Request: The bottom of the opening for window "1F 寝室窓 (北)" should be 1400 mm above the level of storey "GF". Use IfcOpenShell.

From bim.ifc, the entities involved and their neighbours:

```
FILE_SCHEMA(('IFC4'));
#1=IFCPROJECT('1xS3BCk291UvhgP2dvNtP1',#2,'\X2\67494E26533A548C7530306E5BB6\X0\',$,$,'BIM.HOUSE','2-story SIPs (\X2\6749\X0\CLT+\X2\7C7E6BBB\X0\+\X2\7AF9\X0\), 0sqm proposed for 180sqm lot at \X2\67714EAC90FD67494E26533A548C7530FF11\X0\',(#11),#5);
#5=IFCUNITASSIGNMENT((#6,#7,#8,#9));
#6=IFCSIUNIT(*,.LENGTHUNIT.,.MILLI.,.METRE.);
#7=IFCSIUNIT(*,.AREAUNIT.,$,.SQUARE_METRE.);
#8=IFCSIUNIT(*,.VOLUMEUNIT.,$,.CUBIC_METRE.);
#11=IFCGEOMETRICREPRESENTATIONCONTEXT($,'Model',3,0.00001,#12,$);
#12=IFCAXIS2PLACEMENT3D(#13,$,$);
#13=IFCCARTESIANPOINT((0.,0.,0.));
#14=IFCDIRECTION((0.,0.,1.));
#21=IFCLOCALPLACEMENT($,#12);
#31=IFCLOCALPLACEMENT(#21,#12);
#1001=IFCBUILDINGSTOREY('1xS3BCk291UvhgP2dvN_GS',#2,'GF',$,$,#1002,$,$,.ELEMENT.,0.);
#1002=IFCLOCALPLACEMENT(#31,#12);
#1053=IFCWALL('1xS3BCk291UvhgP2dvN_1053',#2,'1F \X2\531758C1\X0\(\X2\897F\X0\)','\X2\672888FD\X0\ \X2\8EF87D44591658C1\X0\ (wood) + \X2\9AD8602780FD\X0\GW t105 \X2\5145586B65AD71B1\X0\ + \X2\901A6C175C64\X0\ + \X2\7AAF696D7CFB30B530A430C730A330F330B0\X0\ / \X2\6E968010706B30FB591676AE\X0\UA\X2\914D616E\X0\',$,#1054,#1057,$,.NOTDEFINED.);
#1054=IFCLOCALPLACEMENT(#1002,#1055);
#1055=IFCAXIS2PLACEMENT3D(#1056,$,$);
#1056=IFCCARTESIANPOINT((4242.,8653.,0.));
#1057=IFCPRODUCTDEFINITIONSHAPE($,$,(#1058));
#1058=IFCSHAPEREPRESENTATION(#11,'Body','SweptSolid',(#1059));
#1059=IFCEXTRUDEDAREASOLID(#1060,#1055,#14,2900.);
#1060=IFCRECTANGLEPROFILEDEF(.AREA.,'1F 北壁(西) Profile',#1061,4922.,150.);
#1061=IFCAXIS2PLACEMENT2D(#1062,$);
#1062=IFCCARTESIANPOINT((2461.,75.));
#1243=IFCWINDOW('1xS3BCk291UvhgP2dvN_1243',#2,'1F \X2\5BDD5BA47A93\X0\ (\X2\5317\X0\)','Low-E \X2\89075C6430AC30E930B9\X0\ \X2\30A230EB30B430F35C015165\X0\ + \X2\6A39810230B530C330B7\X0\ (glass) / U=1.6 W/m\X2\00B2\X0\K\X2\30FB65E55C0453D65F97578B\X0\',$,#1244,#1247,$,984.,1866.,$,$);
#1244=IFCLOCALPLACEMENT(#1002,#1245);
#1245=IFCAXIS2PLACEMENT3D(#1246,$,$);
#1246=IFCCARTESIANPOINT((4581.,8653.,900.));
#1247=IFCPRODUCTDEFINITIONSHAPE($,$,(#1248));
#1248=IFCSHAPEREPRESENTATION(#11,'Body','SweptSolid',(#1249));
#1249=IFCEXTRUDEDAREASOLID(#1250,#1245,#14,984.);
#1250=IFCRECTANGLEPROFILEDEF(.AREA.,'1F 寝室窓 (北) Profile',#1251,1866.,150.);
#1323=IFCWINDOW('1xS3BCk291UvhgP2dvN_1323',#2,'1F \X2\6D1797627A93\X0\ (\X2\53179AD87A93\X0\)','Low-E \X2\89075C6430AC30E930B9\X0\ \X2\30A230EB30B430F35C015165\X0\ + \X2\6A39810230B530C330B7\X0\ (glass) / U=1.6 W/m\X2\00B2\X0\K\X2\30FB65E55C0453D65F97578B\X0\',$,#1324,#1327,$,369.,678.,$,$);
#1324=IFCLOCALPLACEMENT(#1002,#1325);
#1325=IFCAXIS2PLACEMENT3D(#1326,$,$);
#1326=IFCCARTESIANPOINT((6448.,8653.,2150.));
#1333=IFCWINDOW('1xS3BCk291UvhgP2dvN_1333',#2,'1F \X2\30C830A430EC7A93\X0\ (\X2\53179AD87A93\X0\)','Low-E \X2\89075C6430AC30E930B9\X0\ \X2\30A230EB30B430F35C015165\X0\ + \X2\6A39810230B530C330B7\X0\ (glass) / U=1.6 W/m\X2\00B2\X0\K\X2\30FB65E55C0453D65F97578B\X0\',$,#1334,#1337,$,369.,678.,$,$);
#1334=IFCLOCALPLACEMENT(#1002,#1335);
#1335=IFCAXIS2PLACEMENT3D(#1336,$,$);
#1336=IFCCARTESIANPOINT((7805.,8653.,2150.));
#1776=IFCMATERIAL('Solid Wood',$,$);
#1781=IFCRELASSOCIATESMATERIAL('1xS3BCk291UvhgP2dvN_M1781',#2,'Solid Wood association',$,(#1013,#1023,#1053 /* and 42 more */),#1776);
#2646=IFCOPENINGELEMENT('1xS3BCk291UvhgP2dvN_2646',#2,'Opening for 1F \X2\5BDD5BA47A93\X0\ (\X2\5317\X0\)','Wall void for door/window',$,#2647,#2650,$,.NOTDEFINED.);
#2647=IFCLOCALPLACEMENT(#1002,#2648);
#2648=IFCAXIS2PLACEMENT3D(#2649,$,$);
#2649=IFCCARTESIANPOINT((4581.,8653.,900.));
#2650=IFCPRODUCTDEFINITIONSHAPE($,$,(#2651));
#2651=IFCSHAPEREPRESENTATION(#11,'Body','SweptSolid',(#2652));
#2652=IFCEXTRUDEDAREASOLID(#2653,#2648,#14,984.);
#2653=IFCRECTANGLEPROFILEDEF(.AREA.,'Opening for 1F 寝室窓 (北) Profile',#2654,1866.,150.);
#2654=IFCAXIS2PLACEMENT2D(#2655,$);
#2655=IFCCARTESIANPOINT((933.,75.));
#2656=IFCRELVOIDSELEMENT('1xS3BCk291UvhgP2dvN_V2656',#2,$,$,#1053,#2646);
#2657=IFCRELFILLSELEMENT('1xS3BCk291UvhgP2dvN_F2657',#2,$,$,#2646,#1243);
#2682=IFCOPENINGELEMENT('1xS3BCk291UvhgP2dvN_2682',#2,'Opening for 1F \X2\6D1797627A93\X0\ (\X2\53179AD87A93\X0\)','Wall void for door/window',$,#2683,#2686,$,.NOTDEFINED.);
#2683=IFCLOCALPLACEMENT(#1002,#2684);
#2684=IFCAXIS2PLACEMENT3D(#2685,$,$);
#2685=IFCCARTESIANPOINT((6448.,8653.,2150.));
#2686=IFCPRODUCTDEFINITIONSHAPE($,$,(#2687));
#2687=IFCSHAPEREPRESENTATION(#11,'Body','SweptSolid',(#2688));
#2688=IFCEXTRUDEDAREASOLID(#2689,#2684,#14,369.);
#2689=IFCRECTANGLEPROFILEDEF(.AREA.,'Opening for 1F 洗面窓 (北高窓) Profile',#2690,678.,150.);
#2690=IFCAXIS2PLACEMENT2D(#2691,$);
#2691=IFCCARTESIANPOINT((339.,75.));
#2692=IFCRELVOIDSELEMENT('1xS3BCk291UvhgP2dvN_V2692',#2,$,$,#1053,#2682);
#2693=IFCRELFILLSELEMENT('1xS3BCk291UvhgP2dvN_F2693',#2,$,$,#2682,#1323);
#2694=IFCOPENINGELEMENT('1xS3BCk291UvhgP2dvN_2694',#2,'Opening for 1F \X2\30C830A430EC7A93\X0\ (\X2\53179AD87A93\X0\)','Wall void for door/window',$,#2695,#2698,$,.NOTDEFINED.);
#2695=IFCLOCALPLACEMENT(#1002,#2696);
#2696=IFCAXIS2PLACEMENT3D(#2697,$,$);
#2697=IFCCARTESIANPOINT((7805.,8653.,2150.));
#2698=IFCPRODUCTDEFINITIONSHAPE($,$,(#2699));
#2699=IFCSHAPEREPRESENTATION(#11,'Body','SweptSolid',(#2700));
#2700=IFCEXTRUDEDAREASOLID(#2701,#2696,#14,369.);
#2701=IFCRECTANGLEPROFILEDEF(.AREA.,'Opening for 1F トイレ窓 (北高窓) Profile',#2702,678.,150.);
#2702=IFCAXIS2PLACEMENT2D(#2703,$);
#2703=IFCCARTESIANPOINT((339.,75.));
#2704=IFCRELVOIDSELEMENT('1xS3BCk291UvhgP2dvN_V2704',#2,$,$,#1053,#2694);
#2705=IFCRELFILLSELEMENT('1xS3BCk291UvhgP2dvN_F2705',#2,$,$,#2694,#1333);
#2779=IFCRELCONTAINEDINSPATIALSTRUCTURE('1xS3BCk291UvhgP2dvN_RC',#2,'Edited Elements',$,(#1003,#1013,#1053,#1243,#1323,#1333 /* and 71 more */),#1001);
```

```python
import numpy as np
import ifcopenshell
import ifcopenshell.api.geometry
import ifcopenshell.geom
import ifcopenshell.util.element
import ifcopenshell.util.placement
import ifcopenshell.util.shape
import ifcopenshell.util.unit

model = ifcopenshell.open("bim.ifc")
unit_scale = ifcopenshell.util.unit.calculate_unit_scale(model)

window = model.by_guid("1xS3BCk291UvhgP2dvN_1243")
opening = window.FillsVoids[0].RelatingOpeningElement
storey = ifcopenshell.util.element.get_container(window, ifc_class="IfcBuildingStorey")
level = ifcopenshell.util.placement.get_local_placement(storey.ObjectPlacement)[2, 3]

# The opening's origin need not be at the sill, so measure its lowest point.
shape = ifcopenshell.geom.create_shape(ifcopenshell.geom.settings(), opening)
bottom = ifcopenshell.util.shape.get_shape_bottom_elevation(shape, shape.geometry) / unit_scale
dz = level + 1.4 / unit_scale - bottom

shift = np.array([0.0, 0.0, dz])
# The window is not placed relative to its opening, so move both.
for product in (opening, window):
    matrix = ifcopenshell.util.placement.get_local_placement(product.ObjectPlacement)
    matrix[:3, 3] += shift
    ifcopenshell.api.geometry.edit_object_placement(model, product=product, matrix=matrix, is_si=False)

print(f"moved by {dz * unit_scale:+.3f} m")

model.write("bim-out.ifc")
```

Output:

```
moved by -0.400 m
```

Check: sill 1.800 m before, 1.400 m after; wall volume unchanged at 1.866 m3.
